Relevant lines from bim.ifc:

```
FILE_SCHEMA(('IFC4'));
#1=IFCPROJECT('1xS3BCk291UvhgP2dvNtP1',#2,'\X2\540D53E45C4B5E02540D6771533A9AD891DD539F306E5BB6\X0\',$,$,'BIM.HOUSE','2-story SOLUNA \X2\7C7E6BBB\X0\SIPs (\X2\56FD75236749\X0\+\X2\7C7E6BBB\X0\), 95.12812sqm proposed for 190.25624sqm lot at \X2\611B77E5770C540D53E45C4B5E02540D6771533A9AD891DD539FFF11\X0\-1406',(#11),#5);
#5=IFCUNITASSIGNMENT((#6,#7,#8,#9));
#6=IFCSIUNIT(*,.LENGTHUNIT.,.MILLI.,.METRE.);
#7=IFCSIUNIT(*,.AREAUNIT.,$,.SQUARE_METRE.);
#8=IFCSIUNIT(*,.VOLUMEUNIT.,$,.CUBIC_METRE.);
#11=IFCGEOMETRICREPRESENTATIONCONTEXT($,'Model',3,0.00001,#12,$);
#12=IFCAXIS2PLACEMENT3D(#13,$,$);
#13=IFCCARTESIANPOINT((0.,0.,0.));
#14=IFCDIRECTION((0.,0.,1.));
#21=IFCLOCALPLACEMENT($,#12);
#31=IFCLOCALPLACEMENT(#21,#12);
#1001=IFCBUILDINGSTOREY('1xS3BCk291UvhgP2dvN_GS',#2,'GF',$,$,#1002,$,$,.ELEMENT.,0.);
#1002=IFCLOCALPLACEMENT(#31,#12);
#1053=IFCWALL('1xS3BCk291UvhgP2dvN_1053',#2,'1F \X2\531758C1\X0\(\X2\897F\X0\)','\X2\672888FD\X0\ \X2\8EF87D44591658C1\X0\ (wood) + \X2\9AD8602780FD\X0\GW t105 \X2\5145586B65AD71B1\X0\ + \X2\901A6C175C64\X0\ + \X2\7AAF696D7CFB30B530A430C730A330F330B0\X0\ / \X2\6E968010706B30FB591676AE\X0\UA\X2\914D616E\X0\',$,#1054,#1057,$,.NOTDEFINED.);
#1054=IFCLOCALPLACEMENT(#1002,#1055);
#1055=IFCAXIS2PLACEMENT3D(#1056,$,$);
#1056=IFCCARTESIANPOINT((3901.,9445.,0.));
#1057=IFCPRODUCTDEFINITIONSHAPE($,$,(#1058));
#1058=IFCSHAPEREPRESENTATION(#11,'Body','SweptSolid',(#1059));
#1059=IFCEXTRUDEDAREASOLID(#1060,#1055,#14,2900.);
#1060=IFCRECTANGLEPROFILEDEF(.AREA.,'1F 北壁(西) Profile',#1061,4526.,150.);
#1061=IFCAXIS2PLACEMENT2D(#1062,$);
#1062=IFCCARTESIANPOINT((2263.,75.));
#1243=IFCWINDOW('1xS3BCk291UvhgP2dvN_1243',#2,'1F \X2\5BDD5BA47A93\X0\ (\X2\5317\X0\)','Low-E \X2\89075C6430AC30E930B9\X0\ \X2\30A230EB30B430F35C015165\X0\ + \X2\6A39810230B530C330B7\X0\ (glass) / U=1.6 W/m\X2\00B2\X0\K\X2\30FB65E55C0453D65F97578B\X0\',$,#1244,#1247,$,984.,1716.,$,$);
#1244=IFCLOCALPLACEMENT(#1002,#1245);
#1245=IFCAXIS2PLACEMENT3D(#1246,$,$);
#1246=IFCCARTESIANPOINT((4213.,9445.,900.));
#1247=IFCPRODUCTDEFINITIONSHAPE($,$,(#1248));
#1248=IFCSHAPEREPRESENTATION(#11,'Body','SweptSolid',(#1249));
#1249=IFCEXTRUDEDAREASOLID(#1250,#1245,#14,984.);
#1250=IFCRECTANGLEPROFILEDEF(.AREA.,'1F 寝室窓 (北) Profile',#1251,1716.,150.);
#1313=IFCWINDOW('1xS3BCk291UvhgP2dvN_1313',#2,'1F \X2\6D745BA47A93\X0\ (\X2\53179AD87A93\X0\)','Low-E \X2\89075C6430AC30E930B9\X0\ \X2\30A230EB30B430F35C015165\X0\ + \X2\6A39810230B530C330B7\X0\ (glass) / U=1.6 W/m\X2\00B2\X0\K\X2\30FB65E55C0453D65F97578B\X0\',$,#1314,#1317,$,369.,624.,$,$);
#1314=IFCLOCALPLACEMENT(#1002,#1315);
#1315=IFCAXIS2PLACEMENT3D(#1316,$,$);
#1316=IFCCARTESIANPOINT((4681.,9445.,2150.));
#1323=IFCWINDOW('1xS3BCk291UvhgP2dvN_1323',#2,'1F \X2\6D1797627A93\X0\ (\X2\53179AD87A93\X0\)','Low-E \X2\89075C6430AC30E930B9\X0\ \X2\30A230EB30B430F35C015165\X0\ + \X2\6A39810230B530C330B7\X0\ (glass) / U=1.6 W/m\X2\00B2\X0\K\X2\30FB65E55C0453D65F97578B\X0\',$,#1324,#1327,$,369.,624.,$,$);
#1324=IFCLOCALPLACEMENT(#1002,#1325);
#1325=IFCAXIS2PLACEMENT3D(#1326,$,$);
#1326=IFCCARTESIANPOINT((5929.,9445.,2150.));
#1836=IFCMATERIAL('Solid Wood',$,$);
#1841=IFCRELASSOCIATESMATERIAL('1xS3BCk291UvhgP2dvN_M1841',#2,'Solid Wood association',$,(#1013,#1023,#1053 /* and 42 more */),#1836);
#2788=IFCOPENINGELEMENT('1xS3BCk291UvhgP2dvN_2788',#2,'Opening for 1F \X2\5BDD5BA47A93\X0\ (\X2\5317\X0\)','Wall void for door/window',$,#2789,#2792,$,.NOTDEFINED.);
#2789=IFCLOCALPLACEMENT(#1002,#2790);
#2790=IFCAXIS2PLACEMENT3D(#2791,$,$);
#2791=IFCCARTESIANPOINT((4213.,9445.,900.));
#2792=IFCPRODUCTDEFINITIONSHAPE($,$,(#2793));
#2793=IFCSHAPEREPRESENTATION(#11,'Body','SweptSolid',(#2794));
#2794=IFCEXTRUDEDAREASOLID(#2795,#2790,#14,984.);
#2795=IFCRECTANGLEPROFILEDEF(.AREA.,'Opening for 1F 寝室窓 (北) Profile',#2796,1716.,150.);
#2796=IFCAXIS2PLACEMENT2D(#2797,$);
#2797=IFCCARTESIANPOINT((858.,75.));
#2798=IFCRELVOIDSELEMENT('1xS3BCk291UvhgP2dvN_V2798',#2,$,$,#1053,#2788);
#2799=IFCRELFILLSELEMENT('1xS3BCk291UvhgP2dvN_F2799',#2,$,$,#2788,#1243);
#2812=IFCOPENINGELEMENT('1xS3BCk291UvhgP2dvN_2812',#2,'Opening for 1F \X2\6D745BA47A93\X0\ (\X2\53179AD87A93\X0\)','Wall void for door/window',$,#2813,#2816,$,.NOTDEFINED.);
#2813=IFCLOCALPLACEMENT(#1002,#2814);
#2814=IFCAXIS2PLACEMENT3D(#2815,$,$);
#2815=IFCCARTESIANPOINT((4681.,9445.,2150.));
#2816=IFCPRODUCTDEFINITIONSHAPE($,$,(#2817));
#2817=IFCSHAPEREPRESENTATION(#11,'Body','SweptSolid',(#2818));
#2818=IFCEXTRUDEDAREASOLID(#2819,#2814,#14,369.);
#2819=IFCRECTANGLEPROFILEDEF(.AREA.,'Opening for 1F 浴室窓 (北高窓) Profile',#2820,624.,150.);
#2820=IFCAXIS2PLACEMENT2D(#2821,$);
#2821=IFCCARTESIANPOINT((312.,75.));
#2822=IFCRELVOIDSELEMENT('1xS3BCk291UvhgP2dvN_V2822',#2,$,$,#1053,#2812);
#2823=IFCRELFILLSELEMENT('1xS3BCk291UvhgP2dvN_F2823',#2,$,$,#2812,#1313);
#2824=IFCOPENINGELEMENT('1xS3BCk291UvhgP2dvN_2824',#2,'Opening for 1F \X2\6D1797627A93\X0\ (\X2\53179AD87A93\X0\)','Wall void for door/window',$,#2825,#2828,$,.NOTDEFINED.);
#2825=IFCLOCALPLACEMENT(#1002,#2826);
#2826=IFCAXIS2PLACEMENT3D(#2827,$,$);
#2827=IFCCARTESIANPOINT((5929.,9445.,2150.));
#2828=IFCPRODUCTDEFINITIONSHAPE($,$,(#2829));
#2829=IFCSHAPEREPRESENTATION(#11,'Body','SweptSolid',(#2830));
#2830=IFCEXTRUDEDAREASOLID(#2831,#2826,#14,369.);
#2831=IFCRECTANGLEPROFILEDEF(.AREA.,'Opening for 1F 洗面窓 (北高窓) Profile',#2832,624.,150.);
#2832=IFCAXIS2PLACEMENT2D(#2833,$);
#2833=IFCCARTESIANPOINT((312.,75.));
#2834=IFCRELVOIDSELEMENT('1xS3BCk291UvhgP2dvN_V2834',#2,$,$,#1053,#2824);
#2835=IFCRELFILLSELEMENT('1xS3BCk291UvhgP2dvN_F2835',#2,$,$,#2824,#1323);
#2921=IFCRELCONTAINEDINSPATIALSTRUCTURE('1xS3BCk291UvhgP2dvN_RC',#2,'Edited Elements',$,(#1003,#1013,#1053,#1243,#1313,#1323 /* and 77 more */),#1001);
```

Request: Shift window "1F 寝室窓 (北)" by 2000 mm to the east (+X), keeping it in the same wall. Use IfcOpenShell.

```python
import ifcopenshell
import ifcopenshell.api.geometry
import ifcopenshell.util.placement

model = ifcopenshell.open("bim.ifc")

window = model.by_guid("1xS3BCk291UvhgP2dvN_1243")
opening = window.FillsVoids[0].RelatingOpeningElement
wall = opening.VoidsElements[0].RelatingBuildingElement

wall_matrix = ifcopenshell.util.placement.get_local_placement(wall.ObjectPlacement)
shift = wall_matrix[:3, 0] * 2000.0
before = ifcopenshell.util.placement.get_local_placement(window.ObjectPlacement)[:3, 3].copy()

# The window is not placed relative to its opening, so move both.
for product in (opening, window):
    matrix = ifcopenshell.util.placement.get_local_placement(product.ObjectPlacement)
    matrix[:3, 3] += shift
    ifcopenshell.api.geometry.edit_object_placement(model, product=product, matrix=matrix, is_si=False)

after = ifcopenshell.util.placement.get_local_placement(window.ObjectPlacement)[:3, 3]
print("window moved by", (after - before).round(3) + 0.0)

model.write("bim_rev.ifc")
```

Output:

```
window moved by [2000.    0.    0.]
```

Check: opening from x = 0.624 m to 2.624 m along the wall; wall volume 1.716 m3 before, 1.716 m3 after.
